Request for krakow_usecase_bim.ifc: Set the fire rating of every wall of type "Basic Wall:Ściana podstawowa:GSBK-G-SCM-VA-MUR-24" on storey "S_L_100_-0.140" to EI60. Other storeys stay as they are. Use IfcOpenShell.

First a look at what the model holds.

```python
import ifcopenshell
import ifcopenshell.util.element

model = ifcopenshell.open("krakow_usecase_bim.ifc")
print(model.schema)
storey = next(s for s in model.by_type("IfcBuildingStorey") if s.Name == "S_L_100_-0.140")
walls = [e for e in ifcopenshell.util.element.get_decomposition(storey) if e.is_a("IfcWall")]
seen = {}
for e in walls:
    element_type = ifcopenshell.util.element.get_type(e)
    key = (element_type.Name if element_type != e and element_type else None, ifcopenshell.util.element.get_pset(e, "Pset_WallCommon", "FireRating"))
    seen[key] = seen.get(key, 0) + 1
for (name, value), count in sorted(seen.items(), key=str):
    print(count, "x", name, "|", value)
```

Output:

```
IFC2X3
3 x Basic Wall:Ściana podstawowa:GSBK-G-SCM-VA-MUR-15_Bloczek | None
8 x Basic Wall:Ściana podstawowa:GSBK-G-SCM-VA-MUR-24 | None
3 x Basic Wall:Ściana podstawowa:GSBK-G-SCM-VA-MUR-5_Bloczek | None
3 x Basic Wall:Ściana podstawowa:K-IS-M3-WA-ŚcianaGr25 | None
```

```python
import ifcopenshell
import ifcopenshell.api.pset
import ifcopenshell.util.element

model = ifcopenshell.open("krakow_usecase_bim.ifc")

storey = next(s for s in model.by_type("IfcBuildingStorey") if s.Name == "S_L_100_-0.140")
walls = [e for e in ifcopenshell.util.element.get_decomposition(storey) if e.is_a("IfcWall")]

count = 0
for e in walls:
    element_type = ifcopenshell.util.element.get_type(e)
    if element_type in (None, e) or element_type.Name != "Basic Wall:Ściana podstawowa:GSBK-G-SCM-VA-MUR-24":
        continue
    # add_pset returns the element's existing set when there is one.
    pset = ifcopenshell.api.pset.add_pset(model, product=e, name="Pset_WallCommon")
    ifcopenshell.api.pset.edit_pset(model, pset=pset, properties={"FireRating": "EI60"})
    count += 1

print(count, "walls updated")

model.write("krakow_usecase_bim_edited.ifc")
```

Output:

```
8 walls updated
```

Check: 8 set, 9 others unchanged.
